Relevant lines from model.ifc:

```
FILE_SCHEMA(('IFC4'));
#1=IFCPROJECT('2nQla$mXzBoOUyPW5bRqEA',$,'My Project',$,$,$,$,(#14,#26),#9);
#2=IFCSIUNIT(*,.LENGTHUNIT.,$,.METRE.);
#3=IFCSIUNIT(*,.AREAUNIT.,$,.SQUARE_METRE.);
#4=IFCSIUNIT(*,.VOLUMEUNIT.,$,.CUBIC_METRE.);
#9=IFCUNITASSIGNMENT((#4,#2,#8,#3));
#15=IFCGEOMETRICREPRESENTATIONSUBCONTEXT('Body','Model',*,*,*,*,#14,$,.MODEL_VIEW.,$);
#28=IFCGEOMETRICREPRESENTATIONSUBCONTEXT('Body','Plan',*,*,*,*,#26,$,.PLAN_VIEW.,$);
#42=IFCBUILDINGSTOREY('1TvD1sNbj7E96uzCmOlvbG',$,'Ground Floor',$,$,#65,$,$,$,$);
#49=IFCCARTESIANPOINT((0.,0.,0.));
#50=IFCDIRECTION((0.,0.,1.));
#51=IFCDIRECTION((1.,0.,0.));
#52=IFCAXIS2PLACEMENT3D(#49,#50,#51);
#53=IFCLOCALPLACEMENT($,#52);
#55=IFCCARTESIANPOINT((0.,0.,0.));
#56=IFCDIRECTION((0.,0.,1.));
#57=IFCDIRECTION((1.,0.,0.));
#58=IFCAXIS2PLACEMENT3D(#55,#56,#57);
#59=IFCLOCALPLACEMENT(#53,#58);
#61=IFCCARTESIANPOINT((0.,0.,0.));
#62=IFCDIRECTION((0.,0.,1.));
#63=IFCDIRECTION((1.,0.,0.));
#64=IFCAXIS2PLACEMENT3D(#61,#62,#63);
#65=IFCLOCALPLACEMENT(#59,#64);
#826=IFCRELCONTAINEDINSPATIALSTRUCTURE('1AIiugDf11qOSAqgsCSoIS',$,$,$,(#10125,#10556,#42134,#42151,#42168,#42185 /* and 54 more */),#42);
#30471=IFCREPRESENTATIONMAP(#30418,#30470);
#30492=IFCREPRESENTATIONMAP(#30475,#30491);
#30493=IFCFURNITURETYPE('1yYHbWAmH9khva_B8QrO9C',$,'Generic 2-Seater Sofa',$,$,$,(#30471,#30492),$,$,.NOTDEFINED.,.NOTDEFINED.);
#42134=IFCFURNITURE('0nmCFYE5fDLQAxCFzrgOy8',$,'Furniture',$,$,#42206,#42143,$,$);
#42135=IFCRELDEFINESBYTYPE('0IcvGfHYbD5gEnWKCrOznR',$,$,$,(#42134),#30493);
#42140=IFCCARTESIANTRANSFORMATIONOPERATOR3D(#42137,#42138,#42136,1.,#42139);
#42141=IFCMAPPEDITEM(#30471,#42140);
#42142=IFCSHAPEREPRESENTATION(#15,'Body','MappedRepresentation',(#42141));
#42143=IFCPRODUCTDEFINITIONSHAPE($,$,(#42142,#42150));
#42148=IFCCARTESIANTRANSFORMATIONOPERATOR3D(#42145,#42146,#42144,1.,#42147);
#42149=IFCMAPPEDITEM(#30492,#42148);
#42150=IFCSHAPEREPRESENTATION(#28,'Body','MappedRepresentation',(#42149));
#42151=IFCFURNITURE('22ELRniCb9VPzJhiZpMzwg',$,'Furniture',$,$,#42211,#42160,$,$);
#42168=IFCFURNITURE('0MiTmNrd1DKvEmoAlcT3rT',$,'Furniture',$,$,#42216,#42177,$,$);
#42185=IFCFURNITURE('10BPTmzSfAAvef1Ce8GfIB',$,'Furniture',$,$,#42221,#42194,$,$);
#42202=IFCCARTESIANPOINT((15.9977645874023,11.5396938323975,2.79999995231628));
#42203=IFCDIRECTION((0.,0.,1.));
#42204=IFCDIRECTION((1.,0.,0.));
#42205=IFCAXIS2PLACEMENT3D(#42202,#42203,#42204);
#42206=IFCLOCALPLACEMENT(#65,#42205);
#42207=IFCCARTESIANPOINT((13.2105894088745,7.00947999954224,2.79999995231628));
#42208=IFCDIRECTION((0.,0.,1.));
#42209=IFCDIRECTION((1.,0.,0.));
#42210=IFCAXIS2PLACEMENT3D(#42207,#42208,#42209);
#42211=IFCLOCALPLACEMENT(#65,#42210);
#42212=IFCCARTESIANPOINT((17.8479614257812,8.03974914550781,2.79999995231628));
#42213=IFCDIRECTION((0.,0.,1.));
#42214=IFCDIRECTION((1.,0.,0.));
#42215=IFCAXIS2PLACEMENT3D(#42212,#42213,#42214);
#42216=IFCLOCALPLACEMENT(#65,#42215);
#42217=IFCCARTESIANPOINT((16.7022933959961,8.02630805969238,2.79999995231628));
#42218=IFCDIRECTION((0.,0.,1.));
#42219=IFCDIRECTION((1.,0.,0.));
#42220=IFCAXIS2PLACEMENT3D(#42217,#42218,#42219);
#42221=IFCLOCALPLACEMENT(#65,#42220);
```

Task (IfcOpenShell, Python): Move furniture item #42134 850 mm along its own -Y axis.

```python
import ifcopenshell
import ifcopenshell.api.geometry
import ifcopenshell.util.placement

model = ifcopenshell.open("model.ifc")

item = model.by_guid("0nmCFYE5fDLQAxCFzrgOy8")
matrix = ifcopenshell.util.placement.get_local_placement(item.ObjectPlacement)
matrix[:3, 3] -= matrix[:3, 1] * 0.85
ifcopenshell.api.geometry.edit_object_placement(model, product=item, matrix=matrix, is_si=False)

print(ifcopenshell.util.placement.get_local_placement(item.ObjectPlacement).round(3) + 0.0)

model.write("model-out.ifc")
```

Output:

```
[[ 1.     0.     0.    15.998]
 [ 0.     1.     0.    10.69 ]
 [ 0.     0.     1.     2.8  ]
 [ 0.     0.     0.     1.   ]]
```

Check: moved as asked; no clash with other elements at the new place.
